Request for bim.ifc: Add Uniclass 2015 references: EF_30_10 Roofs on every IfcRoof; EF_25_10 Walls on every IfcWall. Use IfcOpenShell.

First a look at what the model holds.

```python
import ifcopenshell

model = ifcopenshell.open("bim.ifc")
print(model.schema)
print("classifications:", [c.Name for c in model.by_type("IfcClassification")])
for ifc_class in ("IfcDoor", "IfcRoof", "IfcStair", "IfcWall", "IfcWindow"):
    print(ifc_class, len(model.by_type(ifc_class)))
```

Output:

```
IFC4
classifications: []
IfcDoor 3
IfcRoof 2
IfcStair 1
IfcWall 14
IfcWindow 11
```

```python
import ifcopenshell
import ifcopenshell.api.classification

model = ifcopenshell.open("bim.ifc")

system = ifcopenshell.api.classification.add_classification(model, classification="Uniclass 2015")

codes = {
    "IfcRoof": ("EF_30_10", "Roofs"),
    "IfcWall": ("EF_25_10", "Walls"),
}
for ifc_class, (code, name) in codes.items():
    products = model.by_type(ifc_class)
    ifcopenshell.api.classification.add_reference(
        model, products=products, classification=system, identification=code, name=name
    )
    print(code, len(products))

model.write("bim-out.ifc")
```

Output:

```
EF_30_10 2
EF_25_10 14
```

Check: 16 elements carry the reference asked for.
